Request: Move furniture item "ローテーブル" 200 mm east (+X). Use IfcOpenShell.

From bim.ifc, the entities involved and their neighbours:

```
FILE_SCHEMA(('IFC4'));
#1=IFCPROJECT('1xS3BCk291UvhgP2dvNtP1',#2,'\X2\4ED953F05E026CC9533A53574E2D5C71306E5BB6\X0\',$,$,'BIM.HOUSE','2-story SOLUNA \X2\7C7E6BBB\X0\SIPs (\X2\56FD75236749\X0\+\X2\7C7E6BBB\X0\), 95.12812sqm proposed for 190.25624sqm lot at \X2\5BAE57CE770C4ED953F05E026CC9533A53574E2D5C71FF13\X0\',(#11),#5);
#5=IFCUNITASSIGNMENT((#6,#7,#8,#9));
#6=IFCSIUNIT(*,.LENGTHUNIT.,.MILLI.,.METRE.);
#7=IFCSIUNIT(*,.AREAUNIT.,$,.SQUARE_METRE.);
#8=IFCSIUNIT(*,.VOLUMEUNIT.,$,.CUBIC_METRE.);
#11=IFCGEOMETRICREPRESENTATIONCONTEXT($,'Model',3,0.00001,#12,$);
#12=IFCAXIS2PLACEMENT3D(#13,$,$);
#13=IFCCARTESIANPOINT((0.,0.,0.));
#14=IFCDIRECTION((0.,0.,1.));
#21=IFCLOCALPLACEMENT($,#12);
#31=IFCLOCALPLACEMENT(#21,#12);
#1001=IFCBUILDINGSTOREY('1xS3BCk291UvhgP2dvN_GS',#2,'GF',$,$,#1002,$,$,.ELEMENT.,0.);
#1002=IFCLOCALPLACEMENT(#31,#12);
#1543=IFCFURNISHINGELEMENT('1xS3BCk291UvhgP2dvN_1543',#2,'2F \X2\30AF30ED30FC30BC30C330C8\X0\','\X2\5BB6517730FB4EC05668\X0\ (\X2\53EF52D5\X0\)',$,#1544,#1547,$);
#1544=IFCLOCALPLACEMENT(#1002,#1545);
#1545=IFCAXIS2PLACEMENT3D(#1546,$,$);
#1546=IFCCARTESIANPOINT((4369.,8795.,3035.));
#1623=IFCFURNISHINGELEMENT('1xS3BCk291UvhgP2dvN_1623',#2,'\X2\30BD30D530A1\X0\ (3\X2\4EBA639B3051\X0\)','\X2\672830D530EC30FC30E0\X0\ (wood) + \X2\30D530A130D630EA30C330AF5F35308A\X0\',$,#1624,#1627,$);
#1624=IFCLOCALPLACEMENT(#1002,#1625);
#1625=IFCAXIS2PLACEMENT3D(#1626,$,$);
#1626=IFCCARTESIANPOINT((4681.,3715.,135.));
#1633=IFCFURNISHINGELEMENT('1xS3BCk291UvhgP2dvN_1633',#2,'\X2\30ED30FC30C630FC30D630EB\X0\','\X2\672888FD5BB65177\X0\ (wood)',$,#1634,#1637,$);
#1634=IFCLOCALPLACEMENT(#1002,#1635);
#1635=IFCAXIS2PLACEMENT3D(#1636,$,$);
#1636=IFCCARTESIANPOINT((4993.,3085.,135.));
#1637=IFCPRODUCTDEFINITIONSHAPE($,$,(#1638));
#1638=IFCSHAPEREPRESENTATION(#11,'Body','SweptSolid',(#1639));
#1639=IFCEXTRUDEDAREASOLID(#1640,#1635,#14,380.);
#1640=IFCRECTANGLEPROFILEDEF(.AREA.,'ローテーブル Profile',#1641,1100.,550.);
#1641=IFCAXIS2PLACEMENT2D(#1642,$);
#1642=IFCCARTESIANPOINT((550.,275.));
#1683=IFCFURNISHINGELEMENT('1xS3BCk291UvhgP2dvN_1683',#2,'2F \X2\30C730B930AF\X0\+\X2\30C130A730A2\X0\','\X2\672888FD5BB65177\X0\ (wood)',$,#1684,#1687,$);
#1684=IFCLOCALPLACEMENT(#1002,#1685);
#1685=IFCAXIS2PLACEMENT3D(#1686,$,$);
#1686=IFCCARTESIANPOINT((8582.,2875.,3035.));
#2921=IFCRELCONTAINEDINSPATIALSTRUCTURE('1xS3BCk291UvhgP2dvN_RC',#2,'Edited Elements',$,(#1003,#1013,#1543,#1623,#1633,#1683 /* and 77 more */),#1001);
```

```python
import ifcopenshell
import ifcopenshell.api.geometry
import ifcopenshell.util.placement
import ifcopenshell.util.unit

model = ifcopenshell.open("bim.ifc")
unit_scale = ifcopenshell.util.unit.calculate_unit_scale(model)

item = model.by_guid("1xS3BCk291UvhgP2dvN_1633")
matrix = ifcopenshell.util.placement.get_local_placement(item.ObjectPlacement)
matrix[0, 3] += 0.2 / unit_scale
ifcopenshell.api.geometry.edit_object_placement(model, product=item, matrix=matrix, is_si=False)

print(ifcopenshell.util.placement.get_local_placement(item.ObjectPlacement).round(3) + 0.0)

model.write("bim_updated.ifc")
```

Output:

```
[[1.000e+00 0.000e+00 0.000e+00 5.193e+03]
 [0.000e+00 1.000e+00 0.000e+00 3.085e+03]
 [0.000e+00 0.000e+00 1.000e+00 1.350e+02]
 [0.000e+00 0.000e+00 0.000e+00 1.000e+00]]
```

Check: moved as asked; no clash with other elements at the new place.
